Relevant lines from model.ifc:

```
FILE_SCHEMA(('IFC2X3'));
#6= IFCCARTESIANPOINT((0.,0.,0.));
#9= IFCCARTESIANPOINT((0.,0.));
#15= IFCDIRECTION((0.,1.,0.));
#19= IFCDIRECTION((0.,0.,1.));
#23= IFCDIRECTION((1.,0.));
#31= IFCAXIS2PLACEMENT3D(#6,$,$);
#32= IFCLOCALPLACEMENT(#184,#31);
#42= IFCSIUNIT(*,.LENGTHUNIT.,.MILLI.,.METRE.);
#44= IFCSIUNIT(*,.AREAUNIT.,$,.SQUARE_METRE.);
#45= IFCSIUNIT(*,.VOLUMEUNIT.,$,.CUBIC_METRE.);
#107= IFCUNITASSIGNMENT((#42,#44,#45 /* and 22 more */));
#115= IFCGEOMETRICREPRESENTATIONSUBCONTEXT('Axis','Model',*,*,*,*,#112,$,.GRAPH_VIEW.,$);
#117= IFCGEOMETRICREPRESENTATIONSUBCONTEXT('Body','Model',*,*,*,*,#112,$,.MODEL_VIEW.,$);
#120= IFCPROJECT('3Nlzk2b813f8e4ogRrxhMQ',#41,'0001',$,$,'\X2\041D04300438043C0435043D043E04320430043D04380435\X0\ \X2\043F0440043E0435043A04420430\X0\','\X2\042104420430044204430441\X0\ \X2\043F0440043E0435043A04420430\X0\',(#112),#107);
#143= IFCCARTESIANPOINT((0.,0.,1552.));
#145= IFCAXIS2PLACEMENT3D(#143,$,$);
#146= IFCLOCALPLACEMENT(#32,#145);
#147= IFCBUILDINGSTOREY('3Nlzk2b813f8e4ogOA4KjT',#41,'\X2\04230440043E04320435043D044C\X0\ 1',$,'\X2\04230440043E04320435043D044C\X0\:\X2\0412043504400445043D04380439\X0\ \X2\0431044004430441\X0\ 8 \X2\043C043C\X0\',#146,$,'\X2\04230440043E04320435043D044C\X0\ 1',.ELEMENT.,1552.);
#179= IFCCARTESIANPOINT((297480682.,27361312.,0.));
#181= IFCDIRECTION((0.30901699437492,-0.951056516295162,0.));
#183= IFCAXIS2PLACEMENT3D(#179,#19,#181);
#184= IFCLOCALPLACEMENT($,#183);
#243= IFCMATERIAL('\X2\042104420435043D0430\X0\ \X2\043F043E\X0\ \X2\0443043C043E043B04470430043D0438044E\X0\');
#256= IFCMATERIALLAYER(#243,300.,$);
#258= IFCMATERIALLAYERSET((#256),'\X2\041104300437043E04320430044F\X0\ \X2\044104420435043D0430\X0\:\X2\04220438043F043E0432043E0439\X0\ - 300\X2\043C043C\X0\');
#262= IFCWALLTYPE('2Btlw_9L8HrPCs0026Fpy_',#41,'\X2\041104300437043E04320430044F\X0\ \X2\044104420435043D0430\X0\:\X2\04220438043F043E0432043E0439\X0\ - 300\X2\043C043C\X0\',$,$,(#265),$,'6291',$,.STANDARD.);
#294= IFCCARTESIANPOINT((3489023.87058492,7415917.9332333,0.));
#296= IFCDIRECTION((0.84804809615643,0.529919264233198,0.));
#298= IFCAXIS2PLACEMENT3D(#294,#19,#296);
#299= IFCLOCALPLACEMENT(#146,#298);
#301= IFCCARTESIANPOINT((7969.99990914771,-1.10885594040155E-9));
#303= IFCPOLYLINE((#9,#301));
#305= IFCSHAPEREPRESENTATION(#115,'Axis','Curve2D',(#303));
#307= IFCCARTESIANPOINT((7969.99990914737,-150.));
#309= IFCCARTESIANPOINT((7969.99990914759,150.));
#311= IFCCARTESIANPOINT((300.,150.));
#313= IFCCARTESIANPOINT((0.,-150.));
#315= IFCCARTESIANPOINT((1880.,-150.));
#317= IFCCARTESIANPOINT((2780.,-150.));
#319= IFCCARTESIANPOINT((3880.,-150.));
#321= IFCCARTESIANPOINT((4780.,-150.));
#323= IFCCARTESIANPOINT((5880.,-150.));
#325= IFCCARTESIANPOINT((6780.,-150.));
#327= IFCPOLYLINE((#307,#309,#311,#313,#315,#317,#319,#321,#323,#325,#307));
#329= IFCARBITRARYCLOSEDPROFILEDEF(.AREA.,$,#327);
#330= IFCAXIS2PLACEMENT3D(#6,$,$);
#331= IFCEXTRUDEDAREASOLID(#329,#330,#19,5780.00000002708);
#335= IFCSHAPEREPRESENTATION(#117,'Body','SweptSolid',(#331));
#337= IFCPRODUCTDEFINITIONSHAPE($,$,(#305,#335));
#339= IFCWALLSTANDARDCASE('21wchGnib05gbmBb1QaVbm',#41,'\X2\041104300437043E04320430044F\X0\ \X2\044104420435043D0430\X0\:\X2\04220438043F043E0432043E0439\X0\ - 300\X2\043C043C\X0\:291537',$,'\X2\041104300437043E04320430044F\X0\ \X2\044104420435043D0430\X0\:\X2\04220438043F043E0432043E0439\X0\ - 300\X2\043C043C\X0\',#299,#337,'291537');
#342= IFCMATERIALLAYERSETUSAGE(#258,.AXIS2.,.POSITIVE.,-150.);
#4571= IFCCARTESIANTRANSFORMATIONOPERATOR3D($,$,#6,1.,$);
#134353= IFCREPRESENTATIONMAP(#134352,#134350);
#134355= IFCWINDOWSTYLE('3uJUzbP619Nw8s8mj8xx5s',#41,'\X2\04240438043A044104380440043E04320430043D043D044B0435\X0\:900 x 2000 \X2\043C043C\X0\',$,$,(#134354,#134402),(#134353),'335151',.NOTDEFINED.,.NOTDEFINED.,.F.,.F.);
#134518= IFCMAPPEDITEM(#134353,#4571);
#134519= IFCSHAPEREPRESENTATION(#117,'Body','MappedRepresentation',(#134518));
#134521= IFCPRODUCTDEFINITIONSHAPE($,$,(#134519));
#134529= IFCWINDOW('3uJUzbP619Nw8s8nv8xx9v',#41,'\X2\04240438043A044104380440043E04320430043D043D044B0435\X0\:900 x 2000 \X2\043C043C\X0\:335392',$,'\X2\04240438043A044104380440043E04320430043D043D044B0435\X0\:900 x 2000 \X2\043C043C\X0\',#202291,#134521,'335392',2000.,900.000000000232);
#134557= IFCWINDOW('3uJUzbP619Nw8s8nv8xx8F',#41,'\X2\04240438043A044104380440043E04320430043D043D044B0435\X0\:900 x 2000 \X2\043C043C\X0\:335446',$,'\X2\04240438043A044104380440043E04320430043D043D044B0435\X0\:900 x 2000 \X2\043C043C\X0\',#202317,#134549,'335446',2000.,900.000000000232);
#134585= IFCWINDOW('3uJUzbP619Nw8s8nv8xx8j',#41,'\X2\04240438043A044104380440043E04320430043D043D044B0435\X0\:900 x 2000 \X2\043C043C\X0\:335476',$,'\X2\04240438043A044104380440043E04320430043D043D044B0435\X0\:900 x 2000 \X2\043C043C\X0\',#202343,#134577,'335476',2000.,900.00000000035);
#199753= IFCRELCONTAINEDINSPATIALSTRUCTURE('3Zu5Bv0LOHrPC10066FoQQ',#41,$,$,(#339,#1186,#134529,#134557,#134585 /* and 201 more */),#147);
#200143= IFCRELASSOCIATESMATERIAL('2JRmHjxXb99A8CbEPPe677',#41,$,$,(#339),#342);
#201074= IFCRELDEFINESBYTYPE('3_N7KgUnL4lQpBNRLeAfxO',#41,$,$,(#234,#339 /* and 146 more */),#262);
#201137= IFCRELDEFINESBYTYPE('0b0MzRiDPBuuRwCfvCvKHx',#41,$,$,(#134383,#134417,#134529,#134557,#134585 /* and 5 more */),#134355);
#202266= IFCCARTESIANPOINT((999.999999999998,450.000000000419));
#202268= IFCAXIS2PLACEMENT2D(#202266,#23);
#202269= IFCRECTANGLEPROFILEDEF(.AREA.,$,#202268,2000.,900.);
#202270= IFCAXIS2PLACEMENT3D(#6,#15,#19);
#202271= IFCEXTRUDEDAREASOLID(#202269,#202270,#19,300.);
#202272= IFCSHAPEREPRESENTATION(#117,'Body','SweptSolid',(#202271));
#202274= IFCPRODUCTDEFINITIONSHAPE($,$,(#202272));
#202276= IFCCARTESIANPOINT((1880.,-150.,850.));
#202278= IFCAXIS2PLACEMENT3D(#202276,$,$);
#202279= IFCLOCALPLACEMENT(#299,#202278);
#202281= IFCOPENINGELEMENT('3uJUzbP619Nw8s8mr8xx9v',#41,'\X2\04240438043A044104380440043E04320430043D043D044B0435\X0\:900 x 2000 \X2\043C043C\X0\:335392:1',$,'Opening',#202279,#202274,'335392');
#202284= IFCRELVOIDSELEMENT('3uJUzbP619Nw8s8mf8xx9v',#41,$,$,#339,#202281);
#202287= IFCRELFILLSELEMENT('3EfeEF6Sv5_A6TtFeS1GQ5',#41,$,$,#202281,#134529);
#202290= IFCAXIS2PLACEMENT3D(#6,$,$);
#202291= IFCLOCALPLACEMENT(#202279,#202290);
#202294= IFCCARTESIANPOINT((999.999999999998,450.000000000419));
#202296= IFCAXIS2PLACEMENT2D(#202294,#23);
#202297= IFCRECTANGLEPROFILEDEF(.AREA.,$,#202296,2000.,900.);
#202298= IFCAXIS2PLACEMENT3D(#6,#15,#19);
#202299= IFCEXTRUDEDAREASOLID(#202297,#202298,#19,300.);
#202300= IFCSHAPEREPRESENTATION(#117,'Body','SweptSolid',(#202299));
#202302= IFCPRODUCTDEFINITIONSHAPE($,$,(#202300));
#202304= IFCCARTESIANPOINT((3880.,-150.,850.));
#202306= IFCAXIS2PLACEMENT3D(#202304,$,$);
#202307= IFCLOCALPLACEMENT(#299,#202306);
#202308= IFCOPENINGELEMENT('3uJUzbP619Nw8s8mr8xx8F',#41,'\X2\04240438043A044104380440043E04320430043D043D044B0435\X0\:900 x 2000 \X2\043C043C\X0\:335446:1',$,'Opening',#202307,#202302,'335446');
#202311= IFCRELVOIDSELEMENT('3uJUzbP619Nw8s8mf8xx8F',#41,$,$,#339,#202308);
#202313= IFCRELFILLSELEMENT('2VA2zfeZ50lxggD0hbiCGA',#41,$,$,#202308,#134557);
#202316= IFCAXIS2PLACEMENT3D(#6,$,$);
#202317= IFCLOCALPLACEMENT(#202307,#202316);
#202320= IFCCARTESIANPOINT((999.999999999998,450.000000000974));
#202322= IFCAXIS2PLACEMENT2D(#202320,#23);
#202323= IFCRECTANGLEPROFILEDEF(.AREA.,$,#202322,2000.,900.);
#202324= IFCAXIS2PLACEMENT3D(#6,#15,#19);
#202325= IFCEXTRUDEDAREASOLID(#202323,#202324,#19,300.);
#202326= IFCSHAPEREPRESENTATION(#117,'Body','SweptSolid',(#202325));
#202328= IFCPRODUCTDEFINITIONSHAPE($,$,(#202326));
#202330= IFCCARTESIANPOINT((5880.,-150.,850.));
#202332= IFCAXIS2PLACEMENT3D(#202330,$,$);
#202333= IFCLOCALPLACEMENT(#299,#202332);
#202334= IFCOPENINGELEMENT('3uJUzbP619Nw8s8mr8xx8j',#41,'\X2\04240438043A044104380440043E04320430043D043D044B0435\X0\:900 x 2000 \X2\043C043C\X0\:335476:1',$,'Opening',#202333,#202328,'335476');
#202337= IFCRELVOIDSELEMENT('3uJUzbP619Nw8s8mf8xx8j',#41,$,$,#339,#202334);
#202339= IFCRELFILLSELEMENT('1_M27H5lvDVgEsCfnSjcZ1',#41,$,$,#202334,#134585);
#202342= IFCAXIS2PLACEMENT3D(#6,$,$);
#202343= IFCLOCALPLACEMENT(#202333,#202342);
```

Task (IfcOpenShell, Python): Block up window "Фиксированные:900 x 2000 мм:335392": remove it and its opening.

```python
import ifcopenshell
import ifcopenshell.api.feature
import ifcopenshell.api.root
import ifcopenshell.geom
import ifcopenshell.util.shape

model = ifcopenshell.open("model.ifc")
settings = ifcopenshell.geom.settings()


def volume(element):
    """Net volume in cubic metres, openings subtracted."""
    shape = ifcopenshell.geom.create_shape(settings, element)
    return ifcopenshell.util.shape.get_volume(shape.geometry)


window = model.by_guid("3uJUzbP619Nw8s8nv8xx9v")
opening = window.FillsVoids[0].RelatingOpeningElement
wall = opening.VoidsElements[0].RelatingBuildingElement
before = volume(wall)

ifcopenshell.api.root.remove_product(model, product=window)
ifcopenshell.api.feature.remove_feature(model, feature=opening)

after = volume(wall)

print(f"wall volume {before:.3f} -> {after:.3f} m3")

model.write("model_rev.ifc")
```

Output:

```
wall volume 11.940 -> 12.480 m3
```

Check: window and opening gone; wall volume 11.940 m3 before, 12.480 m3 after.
